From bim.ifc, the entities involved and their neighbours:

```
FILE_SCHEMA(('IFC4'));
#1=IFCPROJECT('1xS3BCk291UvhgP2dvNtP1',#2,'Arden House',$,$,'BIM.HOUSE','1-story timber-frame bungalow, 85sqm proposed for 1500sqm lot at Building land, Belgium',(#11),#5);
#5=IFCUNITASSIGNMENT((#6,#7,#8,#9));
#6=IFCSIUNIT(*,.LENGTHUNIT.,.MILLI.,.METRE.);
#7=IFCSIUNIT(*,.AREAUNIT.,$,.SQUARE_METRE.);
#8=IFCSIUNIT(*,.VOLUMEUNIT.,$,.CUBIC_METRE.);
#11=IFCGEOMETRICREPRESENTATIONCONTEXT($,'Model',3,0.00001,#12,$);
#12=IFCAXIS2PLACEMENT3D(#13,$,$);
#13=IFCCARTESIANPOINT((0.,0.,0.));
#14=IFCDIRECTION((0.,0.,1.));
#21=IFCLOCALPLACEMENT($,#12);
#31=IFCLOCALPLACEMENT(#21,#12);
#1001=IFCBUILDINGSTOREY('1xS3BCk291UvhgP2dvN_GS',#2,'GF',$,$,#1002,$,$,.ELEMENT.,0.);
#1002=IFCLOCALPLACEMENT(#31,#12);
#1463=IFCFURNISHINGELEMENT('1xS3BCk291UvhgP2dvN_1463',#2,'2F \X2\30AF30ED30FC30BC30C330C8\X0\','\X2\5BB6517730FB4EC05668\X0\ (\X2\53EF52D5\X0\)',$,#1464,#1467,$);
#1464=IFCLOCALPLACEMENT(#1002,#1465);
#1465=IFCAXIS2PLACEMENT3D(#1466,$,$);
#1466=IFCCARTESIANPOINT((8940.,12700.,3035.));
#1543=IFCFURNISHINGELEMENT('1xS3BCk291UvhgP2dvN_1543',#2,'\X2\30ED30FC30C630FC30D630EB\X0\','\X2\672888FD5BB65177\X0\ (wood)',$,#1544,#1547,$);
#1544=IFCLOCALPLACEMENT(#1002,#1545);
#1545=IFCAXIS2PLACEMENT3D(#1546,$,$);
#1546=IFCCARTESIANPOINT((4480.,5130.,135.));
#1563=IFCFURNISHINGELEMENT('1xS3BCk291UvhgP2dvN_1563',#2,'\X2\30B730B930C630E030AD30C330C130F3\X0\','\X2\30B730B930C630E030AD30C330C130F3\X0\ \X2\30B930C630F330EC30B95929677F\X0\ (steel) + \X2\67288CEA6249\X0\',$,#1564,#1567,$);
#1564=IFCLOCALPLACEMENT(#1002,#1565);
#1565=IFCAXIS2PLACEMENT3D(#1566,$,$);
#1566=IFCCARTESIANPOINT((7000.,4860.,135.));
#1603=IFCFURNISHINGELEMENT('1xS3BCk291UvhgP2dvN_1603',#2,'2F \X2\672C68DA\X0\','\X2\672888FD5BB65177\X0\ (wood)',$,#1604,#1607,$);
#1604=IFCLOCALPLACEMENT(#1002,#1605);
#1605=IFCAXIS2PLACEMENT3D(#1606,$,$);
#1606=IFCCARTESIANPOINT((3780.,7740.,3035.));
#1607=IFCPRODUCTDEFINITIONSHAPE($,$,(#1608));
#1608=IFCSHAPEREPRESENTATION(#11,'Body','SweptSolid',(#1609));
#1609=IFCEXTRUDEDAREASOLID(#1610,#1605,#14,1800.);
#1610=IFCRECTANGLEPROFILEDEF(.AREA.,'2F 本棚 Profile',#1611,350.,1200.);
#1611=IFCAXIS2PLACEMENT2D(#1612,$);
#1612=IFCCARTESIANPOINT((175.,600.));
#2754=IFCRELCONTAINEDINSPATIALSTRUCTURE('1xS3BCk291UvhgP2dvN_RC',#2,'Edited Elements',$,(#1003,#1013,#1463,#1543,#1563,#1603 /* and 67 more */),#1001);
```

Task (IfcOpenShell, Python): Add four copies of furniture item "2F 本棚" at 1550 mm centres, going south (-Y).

```python
import numpy as np
import ifcopenshell
import ifcopenshell.api.geometry
import ifcopenshell.api.root
import ifcopenshell.util.element
import ifcopenshell.util.placement
import ifcopenshell.util.unit

model = ifcopenshell.open("bim.ifc")
unit_scale = ifcopenshell.util.unit.calculate_unit_scale(model)


def reuse_history(source, copy):
    """copy_class also copies each property set's owner history, people and application; keep the originals."""
    for rel in copy.IsDefinedBy:
        if rel.is_a("IfcRelDefinesByProperties") and (history := rel.RelatingPropertyDefinition.OwnerHistory):
            rel.RelatingPropertyDefinition.OwnerHistory = source.OwnerHistory
            ifcopenshell.util.element.remove_deep2(model, history)


source = model.by_guid("1xS3BCk291UvhgP2dvN_1603")
base = ifcopenshell.util.placement.get_local_placement(source.ObjectPlacement)
step = np.array([0.0, -1.0, 0.0]) * 1.55 / unit_scale

for i in range(1, 5):
    copy = ifcopenshell.api.root.copy_class(model, product=source)
    copy.Representation = ifcopenshell.util.element.copy_deep(
        model, source.Representation, exclude=["IfcGeometricRepresentationContext", "IfcRepresentationMap"]
    )
    reuse_history(source, copy)
    matrix = base.copy()
    matrix[:3, 3] += i * step
    print("added at", matrix[:3, 3].round(3) + 0.0)
    ifcopenshell.api.geometry.edit_object_placement(model, product=copy, matrix=matrix, is_si=False)

model.write("bim-out.ifc")
```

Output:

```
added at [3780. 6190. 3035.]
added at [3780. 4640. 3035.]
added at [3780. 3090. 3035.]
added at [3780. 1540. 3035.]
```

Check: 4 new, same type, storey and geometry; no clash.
